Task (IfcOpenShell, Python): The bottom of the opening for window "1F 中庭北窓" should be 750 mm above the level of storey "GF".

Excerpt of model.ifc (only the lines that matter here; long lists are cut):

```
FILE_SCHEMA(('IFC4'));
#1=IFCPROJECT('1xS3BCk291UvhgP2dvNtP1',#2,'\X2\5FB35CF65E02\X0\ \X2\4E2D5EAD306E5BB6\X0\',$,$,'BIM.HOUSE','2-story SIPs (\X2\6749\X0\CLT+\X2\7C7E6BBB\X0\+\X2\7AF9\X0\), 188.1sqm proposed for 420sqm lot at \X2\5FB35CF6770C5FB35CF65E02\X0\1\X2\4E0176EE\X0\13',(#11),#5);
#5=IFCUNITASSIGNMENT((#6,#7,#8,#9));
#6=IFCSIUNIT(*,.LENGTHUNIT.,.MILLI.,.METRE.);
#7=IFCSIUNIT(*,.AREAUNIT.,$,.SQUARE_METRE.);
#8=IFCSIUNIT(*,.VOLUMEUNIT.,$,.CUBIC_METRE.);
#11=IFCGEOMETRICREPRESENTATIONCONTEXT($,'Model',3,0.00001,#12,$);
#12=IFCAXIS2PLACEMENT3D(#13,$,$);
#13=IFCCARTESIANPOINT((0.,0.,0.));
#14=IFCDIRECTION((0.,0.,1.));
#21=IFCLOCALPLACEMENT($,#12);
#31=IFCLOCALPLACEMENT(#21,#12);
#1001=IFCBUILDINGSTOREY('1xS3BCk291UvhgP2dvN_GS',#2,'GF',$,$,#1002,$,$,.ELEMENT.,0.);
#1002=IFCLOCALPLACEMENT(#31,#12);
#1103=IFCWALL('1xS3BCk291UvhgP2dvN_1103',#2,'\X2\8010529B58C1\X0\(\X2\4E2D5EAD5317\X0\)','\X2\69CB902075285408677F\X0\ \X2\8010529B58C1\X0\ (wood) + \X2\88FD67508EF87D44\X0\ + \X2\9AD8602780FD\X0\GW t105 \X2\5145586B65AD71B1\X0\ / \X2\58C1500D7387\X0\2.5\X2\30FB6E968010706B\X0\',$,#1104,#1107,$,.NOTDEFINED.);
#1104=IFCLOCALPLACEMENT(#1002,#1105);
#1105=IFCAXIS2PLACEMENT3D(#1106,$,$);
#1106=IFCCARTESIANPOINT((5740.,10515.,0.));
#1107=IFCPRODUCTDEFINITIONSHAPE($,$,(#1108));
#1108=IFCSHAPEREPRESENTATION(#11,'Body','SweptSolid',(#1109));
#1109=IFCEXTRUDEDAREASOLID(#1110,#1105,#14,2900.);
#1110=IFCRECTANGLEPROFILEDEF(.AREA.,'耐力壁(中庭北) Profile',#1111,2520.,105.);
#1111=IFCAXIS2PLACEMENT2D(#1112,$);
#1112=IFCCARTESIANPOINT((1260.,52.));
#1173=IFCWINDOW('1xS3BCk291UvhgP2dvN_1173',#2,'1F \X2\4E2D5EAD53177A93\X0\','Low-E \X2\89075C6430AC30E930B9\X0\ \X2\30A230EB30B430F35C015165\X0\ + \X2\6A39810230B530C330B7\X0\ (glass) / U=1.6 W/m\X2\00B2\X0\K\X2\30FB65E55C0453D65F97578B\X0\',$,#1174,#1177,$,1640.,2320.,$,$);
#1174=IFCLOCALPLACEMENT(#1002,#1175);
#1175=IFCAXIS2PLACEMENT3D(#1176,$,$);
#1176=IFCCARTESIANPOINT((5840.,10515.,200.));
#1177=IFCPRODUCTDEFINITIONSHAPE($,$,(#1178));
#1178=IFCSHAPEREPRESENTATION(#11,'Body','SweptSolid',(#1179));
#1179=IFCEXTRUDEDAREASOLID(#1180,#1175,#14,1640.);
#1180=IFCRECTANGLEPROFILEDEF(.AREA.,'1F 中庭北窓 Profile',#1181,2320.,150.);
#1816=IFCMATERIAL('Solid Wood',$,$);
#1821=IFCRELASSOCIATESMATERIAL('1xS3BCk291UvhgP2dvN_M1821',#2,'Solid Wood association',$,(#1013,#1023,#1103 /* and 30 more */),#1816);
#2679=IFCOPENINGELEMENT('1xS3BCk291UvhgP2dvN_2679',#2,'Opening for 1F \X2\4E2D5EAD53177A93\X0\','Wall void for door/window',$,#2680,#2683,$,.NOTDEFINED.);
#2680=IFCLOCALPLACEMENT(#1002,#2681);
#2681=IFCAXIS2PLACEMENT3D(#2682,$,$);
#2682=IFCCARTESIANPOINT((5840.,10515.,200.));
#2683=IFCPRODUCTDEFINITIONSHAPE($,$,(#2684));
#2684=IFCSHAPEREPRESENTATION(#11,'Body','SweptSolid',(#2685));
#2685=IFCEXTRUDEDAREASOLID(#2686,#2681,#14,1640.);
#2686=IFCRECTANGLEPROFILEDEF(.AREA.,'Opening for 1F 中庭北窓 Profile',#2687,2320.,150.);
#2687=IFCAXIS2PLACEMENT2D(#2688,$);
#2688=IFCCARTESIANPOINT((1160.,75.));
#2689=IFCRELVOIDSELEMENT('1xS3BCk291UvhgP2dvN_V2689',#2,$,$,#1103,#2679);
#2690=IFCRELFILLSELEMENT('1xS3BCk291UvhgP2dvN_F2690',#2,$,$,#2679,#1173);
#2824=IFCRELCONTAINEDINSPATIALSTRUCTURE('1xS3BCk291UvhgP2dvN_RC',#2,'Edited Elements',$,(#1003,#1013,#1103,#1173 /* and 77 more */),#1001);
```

```python
import numpy as np
import ifcopenshell
import ifcopenshell.api.geometry
import ifcopenshell.geom
import ifcopenshell.util.element
import ifcopenshell.util.placement
import ifcopenshell.util.shape
import ifcopenshell.util.unit

model = ifcopenshell.open("model.ifc")
unit_scale = ifcopenshell.util.unit.calculate_unit_scale(model)

window = model.by_guid("1xS3BCk291UvhgP2dvN_1173")
opening = window.FillsVoids[0].RelatingOpeningElement
storey = ifcopenshell.util.element.get_container(window, ifc_class="IfcBuildingStorey")
level = ifcopenshell.util.placement.get_local_placement(storey.ObjectPlacement)[2, 3]

# The opening's origin need not be at the sill, so measure its lowest point.
shape = ifcopenshell.geom.create_shape(ifcopenshell.geom.settings(), opening)
bottom = ifcopenshell.util.shape.get_shape_bottom_elevation(shape, shape.geometry) / unit_scale
dz = level + 750.0 - bottom

shift = np.array([0.0, 0.0, dz])
# The window is not placed relative to its opening, so move both.
for product in (opening, window):
    matrix = ifcopenshell.util.placement.get_local_placement(product.ObjectPlacement)
    matrix[:3, 3] += shift
    ifcopenshell.api.geometry.edit_object_placement(model, product=product, matrix=matrix, is_si=False)

print(f"moved by {dz * unit_scale:+.3f} m")

model.write("model-out.ifc")
```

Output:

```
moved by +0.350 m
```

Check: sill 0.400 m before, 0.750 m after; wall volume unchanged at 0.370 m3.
